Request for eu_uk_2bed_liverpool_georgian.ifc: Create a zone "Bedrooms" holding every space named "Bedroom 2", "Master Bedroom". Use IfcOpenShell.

First a look at what the model holds.

```python
import ifcopenshell

model = ifcopenshell.open("eu_uk_2bed_liverpool_georgian.ifc")
print(model.schema)
seen = {}
for space in model.by_type("IfcSpace"):
    seen[space.LongName] = seen.get(space.LongName, 0) + 1
for name, count in sorted(seen.items(), key=str):
    print(count, "x", name)
print("zones:", [z.Name for z in model.by_type("IfcZone")][:20])
```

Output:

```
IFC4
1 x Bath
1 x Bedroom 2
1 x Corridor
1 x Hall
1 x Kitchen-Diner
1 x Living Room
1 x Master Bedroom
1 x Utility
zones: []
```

```python
import ifcopenshell
import ifcopenshell.api.group
import ifcopenshell.api.root

model = ifcopenshell.open("eu_uk_2bed_liverpool_georgian.ifc")

names = {"Bedroom 2", "Master Bedroom"}
spaces = [s for s in model.by_type("IfcSpace") if s.LongName in names]

zone = ifcopenshell.api.root.create_entity(model, ifc_class="IfcZone", name="Bedrooms")
ifcopenshell.api.group.assign_group(model, products=spaces, group=zone)
print(len(spaces), "spaces in", zone.Name)

model.write("eu_uk_2bed_liverpool_georgian-out.ifc")
```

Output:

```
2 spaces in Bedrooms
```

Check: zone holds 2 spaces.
